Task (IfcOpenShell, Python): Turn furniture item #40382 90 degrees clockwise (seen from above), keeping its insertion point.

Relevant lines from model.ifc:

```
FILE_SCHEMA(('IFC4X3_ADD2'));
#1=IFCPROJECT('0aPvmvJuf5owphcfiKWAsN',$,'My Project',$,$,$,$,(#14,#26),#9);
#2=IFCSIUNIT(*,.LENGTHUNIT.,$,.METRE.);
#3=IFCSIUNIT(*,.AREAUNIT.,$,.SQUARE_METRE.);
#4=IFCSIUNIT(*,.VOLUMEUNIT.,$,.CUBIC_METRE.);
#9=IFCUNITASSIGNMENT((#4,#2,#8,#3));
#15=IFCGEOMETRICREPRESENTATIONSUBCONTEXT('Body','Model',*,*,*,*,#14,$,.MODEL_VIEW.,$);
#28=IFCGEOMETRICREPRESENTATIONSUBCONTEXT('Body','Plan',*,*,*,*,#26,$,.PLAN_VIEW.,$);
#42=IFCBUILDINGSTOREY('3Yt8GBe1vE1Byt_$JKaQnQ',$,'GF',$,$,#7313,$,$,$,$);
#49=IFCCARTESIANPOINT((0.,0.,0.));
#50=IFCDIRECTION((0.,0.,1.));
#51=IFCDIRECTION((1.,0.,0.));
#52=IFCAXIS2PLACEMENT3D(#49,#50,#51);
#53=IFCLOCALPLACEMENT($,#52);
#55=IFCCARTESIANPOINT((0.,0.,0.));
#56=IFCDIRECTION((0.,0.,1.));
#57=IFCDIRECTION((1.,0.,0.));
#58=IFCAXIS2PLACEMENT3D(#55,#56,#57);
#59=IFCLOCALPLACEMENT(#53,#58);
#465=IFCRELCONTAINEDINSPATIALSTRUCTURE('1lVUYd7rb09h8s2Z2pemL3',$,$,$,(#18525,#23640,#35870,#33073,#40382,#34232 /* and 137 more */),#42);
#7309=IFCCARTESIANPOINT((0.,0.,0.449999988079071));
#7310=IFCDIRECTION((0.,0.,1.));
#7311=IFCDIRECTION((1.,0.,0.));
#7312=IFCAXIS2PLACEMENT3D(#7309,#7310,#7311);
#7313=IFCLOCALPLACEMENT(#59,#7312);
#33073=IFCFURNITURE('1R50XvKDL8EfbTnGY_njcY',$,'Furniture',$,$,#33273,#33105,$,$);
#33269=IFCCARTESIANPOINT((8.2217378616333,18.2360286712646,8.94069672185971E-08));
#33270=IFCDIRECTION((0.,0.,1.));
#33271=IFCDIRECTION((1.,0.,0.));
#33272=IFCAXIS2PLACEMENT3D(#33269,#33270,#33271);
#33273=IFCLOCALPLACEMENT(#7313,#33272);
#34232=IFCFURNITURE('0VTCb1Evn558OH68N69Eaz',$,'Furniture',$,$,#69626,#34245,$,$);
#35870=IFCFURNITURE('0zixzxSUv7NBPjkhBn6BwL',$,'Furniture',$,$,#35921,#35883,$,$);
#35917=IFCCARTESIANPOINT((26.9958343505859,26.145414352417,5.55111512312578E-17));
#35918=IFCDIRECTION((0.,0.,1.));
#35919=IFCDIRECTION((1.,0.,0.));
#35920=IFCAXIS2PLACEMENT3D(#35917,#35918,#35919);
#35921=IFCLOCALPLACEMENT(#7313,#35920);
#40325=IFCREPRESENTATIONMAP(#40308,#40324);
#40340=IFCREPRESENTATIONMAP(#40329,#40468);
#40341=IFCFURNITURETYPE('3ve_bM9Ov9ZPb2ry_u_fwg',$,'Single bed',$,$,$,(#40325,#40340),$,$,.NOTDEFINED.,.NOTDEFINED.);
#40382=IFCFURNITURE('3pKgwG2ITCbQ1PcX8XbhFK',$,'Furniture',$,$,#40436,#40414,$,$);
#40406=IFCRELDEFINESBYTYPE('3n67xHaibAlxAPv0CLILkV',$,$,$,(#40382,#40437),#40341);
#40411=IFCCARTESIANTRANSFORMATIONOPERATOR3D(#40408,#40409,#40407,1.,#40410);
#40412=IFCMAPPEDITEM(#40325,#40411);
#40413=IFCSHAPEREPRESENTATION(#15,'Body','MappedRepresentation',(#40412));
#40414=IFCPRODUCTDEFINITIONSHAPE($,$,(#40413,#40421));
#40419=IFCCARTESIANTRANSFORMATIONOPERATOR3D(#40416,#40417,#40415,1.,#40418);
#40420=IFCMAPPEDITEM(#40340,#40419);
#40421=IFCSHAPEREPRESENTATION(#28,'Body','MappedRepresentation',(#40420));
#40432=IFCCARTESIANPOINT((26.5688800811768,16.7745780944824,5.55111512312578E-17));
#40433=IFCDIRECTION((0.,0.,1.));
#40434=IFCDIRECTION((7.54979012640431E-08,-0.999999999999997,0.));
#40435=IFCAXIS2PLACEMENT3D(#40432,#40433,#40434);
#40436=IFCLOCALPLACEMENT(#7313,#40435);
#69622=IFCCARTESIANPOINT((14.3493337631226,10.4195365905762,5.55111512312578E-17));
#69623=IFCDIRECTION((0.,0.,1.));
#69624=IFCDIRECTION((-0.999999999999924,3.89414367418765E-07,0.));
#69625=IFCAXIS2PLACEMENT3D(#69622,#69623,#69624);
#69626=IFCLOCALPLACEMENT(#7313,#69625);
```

```python
import ifcopenshell
import ifcopenshell.api.geometry
import ifcopenshell.util.placement

model = ifcopenshell.open("model.ifc")

item = model.by_id(40382)
matrix = ifcopenshell.util.placement.get_local_placement(item.ObjectPlacement)
matrix = matrix @ ifcopenshell.util.placement.rotation(-90, "Z")
ifcopenshell.api.geometry.edit_object_placement(model, product=item, matrix=matrix, is_si=False)

print(ifcopenshell.util.placement.get_local_placement(item.ObjectPlacement).round(3) + 0.0)

model.write("model_updated.ifc")
```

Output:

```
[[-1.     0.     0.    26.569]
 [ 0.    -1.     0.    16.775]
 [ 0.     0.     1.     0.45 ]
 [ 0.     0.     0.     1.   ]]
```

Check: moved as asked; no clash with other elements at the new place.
